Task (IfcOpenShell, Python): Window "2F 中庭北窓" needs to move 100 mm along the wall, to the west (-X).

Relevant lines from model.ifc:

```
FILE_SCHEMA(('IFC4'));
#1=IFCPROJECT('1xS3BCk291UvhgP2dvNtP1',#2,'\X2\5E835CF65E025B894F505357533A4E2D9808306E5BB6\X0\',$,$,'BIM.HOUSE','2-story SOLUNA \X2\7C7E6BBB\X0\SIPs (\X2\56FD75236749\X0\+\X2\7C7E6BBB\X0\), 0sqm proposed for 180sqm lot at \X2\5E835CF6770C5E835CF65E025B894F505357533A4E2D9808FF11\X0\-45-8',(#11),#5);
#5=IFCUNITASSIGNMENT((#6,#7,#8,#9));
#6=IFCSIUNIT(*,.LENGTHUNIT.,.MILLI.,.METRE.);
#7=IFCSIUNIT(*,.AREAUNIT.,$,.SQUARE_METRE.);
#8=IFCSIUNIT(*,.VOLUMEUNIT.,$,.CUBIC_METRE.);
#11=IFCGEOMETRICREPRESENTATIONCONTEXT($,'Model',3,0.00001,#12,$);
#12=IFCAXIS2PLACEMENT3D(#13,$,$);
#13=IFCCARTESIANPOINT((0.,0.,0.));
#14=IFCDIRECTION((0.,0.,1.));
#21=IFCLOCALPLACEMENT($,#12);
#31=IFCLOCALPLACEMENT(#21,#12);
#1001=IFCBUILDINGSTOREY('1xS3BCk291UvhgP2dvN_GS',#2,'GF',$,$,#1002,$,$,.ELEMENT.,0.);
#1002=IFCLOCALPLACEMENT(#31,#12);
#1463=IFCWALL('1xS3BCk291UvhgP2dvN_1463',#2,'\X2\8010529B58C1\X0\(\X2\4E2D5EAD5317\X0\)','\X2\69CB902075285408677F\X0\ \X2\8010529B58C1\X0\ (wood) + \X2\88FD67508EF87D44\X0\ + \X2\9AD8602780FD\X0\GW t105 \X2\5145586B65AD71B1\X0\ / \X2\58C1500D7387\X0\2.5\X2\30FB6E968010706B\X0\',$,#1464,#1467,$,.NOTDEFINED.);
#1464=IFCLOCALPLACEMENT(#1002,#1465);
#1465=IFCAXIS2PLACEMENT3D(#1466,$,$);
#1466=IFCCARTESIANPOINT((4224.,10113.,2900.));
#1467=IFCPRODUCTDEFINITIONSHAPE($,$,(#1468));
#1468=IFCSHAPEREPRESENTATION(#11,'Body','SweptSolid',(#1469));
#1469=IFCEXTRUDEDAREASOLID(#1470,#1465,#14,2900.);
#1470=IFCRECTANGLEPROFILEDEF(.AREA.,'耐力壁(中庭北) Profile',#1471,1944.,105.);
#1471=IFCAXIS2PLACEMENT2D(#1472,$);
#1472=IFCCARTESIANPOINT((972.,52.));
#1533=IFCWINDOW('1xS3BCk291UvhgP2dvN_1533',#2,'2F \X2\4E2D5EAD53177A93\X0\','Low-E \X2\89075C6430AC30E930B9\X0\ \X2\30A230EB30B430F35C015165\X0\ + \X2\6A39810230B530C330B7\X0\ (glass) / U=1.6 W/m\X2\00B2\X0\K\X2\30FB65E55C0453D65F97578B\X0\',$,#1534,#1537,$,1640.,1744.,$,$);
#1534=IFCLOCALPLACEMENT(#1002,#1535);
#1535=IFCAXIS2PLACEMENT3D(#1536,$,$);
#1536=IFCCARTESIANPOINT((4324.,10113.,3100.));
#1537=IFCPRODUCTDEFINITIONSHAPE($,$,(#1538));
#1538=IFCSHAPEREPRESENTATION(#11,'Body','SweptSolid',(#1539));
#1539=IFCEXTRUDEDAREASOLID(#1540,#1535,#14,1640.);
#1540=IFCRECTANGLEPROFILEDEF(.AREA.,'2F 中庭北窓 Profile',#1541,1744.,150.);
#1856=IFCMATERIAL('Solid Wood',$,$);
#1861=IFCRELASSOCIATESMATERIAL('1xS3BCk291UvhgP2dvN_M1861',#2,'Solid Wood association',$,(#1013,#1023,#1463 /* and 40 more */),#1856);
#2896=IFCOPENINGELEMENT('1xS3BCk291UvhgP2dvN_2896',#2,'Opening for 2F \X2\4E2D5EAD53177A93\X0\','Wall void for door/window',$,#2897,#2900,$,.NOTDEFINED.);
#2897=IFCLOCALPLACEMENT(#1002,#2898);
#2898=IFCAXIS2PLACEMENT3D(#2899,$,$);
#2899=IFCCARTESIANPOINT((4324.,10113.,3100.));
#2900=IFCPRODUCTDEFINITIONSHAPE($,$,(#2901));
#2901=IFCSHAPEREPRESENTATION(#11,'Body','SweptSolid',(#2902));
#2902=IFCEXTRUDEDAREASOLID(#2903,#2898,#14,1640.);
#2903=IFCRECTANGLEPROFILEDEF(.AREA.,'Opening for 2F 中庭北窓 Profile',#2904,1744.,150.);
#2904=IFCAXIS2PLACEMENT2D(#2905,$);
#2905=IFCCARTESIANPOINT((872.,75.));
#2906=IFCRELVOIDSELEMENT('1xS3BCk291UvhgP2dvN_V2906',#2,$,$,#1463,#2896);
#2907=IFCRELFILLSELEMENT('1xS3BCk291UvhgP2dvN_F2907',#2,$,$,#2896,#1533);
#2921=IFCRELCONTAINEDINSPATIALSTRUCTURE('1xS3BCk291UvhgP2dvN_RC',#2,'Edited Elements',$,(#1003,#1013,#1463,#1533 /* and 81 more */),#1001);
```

```python
import ifcopenshell
import ifcopenshell.api.geometry
import ifcopenshell.util.placement
import ifcopenshell.util.unit

model = ifcopenshell.open("model.ifc")
unit_scale = ifcopenshell.util.unit.calculate_unit_scale(model)

window = model.by_id(1533)
opening = window.FillsVoids[0].RelatingOpeningElement
wall = opening.VoidsElements[0].RelatingBuildingElement

wall_matrix = ifcopenshell.util.placement.get_local_placement(wall.ObjectPlacement)
shift = wall_matrix[:3, 0] * -0.1 / unit_scale
before = ifcopenshell.util.placement.get_local_placement(window.ObjectPlacement)[:3, 3].copy()

# The window is not placed relative to its opening, so move both.
for product in (opening, window):
    matrix = ifcopenshell.util.placement.get_local_placement(product.ObjectPlacement)
    matrix[:3, 3] += shift
    ifcopenshell.api.geometry.edit_object_placement(model, product=product, matrix=matrix, is_si=False)

after = ifcopenshell.util.placement.get_local_placement(window.ObjectPlacement)[:3, 3]
print("window moved by", (after - before).round(3) + 0.0)

model.write("model_updated.ifc")
```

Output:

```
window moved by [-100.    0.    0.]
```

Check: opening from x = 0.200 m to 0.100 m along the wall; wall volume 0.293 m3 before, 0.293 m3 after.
